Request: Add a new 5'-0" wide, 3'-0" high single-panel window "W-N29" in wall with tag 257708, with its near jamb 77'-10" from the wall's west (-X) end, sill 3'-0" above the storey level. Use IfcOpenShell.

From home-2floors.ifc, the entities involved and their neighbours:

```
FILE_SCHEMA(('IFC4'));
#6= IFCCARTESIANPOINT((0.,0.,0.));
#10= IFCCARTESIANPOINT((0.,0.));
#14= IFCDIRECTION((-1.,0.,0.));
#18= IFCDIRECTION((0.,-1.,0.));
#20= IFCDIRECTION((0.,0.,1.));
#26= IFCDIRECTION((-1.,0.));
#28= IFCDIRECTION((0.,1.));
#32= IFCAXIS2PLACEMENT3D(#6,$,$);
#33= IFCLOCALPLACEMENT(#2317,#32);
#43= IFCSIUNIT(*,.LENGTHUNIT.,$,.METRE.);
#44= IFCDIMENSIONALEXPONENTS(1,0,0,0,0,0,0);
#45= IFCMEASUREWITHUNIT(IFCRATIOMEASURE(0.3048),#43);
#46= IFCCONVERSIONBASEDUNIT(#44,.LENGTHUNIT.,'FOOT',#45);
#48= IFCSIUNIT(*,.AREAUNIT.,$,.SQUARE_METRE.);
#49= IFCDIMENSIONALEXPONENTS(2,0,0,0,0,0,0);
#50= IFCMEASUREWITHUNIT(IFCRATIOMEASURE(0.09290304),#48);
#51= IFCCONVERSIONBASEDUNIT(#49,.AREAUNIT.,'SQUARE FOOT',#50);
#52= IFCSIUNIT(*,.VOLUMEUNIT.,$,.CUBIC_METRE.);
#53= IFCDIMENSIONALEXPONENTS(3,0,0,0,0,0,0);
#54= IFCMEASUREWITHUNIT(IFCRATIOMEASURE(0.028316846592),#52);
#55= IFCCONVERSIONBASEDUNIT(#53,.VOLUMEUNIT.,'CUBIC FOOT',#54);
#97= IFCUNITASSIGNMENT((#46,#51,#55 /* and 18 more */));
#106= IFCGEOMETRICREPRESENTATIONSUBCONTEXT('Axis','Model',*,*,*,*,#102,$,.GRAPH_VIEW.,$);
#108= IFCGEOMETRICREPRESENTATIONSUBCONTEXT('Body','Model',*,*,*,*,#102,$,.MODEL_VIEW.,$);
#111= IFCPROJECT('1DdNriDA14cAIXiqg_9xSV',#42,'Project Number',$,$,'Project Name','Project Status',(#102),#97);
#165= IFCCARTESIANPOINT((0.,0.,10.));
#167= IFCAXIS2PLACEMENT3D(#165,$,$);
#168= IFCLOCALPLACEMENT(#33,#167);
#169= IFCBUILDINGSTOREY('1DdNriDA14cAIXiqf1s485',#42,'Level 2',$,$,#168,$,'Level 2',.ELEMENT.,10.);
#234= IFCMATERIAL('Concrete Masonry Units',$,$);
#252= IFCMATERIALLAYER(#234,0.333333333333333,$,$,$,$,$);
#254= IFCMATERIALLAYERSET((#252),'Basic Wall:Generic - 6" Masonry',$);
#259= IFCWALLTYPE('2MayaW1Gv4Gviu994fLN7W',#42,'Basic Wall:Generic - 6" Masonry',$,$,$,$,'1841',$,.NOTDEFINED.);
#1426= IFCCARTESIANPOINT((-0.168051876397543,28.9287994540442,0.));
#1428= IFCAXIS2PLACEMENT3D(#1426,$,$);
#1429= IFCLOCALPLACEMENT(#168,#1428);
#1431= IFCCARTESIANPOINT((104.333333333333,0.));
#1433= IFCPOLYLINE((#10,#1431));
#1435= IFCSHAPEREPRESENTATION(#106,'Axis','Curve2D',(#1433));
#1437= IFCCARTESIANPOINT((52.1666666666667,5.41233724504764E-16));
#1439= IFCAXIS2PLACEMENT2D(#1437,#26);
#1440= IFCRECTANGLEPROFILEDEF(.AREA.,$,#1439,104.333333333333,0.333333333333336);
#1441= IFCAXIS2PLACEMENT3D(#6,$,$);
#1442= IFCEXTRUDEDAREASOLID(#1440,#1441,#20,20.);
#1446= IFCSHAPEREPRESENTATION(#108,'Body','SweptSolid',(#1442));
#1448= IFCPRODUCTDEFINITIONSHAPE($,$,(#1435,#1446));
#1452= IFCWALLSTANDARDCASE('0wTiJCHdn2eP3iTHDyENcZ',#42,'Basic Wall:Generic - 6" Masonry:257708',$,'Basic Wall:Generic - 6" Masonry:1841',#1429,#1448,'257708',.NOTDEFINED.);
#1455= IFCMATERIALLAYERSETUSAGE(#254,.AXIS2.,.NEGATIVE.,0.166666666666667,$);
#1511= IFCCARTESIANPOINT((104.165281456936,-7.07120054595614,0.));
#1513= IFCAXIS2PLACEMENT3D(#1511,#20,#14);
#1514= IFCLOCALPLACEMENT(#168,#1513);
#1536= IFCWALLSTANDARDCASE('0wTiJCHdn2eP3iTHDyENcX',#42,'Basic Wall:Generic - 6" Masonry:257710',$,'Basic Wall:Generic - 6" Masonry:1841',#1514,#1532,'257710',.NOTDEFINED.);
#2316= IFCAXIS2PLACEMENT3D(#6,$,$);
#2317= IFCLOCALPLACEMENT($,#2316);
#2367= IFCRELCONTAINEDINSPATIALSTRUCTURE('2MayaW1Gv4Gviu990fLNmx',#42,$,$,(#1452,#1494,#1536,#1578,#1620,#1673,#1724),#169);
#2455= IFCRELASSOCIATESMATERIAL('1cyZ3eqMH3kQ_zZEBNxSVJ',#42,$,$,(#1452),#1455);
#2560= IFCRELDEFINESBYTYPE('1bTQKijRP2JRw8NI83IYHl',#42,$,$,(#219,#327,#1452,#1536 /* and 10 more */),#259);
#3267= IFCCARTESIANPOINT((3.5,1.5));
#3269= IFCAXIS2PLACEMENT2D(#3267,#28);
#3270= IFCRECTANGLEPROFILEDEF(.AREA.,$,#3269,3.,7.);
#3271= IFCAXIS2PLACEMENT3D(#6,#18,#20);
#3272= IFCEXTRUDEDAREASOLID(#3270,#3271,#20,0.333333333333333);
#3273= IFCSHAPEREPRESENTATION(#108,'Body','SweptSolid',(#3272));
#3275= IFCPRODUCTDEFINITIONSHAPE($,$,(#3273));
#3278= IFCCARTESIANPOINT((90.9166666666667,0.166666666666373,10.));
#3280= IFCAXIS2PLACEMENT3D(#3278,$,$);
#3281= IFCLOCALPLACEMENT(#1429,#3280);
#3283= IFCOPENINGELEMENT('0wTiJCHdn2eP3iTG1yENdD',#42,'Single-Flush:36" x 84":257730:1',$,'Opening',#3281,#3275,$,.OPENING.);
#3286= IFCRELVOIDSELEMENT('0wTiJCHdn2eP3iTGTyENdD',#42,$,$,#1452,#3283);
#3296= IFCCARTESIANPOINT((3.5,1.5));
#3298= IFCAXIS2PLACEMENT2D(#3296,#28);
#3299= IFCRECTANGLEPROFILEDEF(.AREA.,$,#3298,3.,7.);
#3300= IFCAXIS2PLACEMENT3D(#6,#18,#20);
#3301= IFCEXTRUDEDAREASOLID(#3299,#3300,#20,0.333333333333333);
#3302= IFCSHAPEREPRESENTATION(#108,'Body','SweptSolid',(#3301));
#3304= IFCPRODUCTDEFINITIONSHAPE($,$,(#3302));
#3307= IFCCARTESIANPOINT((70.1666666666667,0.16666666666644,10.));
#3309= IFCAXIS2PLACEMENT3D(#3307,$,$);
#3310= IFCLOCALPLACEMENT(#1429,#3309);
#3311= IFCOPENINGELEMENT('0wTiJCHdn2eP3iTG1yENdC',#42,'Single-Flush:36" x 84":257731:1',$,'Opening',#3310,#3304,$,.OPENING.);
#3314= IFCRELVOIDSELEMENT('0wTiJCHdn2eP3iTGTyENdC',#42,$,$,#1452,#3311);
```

```python
import numpy as np
import ifcopenshell
import ifcopenshell.api.feature
import ifcopenshell.api.geometry
import ifcopenshell.api.root
import ifcopenshell.api.spatial
import ifcopenshell.geom
import ifcopenshell.util.element
import ifcopenshell.util.placement
import ifcopenshell.util.representation
import ifcopenshell.util.shape
import ifcopenshell.util.unit

model = ifcopenshell.open("home-2floors.ifc")
unit_scale = ifcopenshell.util.unit.calculate_unit_scale(model)
settings = ifcopenshell.geom.settings()


def volume(element):
    """Net volume in cubic metres, openings subtracted."""
    shape = ifcopenshell.geom.create_shape(settings, element)
    return ifcopenshell.util.shape.get_volume(shape.geometry)


wall = model.by_guid("0wTiJCHdn2eP3iTHDyENcZ")
storey = ifcopenshell.util.element.get_container(wall, ifc_class="IfcBuildingStorey")
context = ifcopenshell.util.representation.get_context(model, "Model", "Body", "MODEL_VIEW")
before = volume(wall)

width, height, from_end, sill = 1.524, 0.9144, 23.7236, 0.9144  # metres

# The wall runs along its own X axis, and the end named is its -X end.
wall_shape = ifcopenshell.geom.create_shape(settings, wall)
x, y, z = ifcopenshell.util.shape.get_vertices(wall_shape.geometry).T
start = x.min() + from_end
face, thickness = float(y.min()), float(y.max() - y.min())
wall_matrix = ifcopenshell.util.placement.get_local_placement(wall.ObjectPlacement)
level = ifcopenshell.util.placement.get_local_placement(storey.ObjectPlacement)[2, 3]


def in_wall(x, y):
    """Placement at x, y metres in the wall's axes, at sill height."""
    matrix = wall_matrix.copy()
    matrix[:, 3] = wall_matrix @ np.array([x / unit_scale, y / unit_scale, 0.0, 1.0])
    matrix[2, 3] = level + sill / unit_scale
    return matrix


# Opening: a box that overshoots both wall faces by 50 mm.
opening = ifcopenshell.api.root.create_entity(model, ifc_class="IfcOpeningElement", predefined_type="OPENING")
box = ifcopenshell.api.geometry.add_wall_representation(
    model, context=context, length=width, height=height, thickness=thickness + 0.1
)
ifcopenshell.api.geometry.assign_representation(model, product=opening, representation=box)
ifcopenshell.api.geometry.edit_object_placement(model, product=opening, matrix=in_wall(start, face - 0.05), is_si=False)
ifcopenshell.api.feature.add_feature(model, feature=opening, element=wall)

window = ifcopenshell.api.root.create_entity(model, ifc_class="IfcWindow", name="W-N29", predefined_type="WINDOW")
window.OverallWidth, window.OverallHeight = width / unit_scale, height / unit_scale
window.PartitioningType = "SINGLE_PANEL"
body = ifcopenshell.api.geometry.add_window_representation(
    model,
    context=context,
    overall_width=window.OverallWidth,
    overall_height=window.OverallHeight,
    partition_type="SINGLE_PANEL",
)
ifcopenshell.api.geometry.assign_representation(model, product=window, representation=body)
ifcopenshell.api.spatial.assign_container(model, products=[window], relating_structure=storey)
ifcopenshell.api.feature.add_filling(model, opening=opening, element=window)

# Centre the window in the wall's thickness.
ifcopenshell.api.geometry.edit_object_placement(model, product=window, matrix=in_wall(start, face), is_si=False)
window_shape = ifcopenshell.geom.create_shape(settings, window)
depth = ifcopenshell.util.shape.get_vertices(window_shape.geometry)[:, 1]
offset = face + thickness / 2 - (depth.min() + depth.max()) / 2
ifcopenshell.api.geometry.edit_object_placement(model, product=window, matrix=in_wall(start, offset), is_si=False)

after = volume(wall)

print(f"wall volume {before:.3f} -> {after:.3f} m3")

model.write("home-2floors_v2.ifc")
```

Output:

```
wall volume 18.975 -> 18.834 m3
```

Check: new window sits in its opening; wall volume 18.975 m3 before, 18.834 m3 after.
